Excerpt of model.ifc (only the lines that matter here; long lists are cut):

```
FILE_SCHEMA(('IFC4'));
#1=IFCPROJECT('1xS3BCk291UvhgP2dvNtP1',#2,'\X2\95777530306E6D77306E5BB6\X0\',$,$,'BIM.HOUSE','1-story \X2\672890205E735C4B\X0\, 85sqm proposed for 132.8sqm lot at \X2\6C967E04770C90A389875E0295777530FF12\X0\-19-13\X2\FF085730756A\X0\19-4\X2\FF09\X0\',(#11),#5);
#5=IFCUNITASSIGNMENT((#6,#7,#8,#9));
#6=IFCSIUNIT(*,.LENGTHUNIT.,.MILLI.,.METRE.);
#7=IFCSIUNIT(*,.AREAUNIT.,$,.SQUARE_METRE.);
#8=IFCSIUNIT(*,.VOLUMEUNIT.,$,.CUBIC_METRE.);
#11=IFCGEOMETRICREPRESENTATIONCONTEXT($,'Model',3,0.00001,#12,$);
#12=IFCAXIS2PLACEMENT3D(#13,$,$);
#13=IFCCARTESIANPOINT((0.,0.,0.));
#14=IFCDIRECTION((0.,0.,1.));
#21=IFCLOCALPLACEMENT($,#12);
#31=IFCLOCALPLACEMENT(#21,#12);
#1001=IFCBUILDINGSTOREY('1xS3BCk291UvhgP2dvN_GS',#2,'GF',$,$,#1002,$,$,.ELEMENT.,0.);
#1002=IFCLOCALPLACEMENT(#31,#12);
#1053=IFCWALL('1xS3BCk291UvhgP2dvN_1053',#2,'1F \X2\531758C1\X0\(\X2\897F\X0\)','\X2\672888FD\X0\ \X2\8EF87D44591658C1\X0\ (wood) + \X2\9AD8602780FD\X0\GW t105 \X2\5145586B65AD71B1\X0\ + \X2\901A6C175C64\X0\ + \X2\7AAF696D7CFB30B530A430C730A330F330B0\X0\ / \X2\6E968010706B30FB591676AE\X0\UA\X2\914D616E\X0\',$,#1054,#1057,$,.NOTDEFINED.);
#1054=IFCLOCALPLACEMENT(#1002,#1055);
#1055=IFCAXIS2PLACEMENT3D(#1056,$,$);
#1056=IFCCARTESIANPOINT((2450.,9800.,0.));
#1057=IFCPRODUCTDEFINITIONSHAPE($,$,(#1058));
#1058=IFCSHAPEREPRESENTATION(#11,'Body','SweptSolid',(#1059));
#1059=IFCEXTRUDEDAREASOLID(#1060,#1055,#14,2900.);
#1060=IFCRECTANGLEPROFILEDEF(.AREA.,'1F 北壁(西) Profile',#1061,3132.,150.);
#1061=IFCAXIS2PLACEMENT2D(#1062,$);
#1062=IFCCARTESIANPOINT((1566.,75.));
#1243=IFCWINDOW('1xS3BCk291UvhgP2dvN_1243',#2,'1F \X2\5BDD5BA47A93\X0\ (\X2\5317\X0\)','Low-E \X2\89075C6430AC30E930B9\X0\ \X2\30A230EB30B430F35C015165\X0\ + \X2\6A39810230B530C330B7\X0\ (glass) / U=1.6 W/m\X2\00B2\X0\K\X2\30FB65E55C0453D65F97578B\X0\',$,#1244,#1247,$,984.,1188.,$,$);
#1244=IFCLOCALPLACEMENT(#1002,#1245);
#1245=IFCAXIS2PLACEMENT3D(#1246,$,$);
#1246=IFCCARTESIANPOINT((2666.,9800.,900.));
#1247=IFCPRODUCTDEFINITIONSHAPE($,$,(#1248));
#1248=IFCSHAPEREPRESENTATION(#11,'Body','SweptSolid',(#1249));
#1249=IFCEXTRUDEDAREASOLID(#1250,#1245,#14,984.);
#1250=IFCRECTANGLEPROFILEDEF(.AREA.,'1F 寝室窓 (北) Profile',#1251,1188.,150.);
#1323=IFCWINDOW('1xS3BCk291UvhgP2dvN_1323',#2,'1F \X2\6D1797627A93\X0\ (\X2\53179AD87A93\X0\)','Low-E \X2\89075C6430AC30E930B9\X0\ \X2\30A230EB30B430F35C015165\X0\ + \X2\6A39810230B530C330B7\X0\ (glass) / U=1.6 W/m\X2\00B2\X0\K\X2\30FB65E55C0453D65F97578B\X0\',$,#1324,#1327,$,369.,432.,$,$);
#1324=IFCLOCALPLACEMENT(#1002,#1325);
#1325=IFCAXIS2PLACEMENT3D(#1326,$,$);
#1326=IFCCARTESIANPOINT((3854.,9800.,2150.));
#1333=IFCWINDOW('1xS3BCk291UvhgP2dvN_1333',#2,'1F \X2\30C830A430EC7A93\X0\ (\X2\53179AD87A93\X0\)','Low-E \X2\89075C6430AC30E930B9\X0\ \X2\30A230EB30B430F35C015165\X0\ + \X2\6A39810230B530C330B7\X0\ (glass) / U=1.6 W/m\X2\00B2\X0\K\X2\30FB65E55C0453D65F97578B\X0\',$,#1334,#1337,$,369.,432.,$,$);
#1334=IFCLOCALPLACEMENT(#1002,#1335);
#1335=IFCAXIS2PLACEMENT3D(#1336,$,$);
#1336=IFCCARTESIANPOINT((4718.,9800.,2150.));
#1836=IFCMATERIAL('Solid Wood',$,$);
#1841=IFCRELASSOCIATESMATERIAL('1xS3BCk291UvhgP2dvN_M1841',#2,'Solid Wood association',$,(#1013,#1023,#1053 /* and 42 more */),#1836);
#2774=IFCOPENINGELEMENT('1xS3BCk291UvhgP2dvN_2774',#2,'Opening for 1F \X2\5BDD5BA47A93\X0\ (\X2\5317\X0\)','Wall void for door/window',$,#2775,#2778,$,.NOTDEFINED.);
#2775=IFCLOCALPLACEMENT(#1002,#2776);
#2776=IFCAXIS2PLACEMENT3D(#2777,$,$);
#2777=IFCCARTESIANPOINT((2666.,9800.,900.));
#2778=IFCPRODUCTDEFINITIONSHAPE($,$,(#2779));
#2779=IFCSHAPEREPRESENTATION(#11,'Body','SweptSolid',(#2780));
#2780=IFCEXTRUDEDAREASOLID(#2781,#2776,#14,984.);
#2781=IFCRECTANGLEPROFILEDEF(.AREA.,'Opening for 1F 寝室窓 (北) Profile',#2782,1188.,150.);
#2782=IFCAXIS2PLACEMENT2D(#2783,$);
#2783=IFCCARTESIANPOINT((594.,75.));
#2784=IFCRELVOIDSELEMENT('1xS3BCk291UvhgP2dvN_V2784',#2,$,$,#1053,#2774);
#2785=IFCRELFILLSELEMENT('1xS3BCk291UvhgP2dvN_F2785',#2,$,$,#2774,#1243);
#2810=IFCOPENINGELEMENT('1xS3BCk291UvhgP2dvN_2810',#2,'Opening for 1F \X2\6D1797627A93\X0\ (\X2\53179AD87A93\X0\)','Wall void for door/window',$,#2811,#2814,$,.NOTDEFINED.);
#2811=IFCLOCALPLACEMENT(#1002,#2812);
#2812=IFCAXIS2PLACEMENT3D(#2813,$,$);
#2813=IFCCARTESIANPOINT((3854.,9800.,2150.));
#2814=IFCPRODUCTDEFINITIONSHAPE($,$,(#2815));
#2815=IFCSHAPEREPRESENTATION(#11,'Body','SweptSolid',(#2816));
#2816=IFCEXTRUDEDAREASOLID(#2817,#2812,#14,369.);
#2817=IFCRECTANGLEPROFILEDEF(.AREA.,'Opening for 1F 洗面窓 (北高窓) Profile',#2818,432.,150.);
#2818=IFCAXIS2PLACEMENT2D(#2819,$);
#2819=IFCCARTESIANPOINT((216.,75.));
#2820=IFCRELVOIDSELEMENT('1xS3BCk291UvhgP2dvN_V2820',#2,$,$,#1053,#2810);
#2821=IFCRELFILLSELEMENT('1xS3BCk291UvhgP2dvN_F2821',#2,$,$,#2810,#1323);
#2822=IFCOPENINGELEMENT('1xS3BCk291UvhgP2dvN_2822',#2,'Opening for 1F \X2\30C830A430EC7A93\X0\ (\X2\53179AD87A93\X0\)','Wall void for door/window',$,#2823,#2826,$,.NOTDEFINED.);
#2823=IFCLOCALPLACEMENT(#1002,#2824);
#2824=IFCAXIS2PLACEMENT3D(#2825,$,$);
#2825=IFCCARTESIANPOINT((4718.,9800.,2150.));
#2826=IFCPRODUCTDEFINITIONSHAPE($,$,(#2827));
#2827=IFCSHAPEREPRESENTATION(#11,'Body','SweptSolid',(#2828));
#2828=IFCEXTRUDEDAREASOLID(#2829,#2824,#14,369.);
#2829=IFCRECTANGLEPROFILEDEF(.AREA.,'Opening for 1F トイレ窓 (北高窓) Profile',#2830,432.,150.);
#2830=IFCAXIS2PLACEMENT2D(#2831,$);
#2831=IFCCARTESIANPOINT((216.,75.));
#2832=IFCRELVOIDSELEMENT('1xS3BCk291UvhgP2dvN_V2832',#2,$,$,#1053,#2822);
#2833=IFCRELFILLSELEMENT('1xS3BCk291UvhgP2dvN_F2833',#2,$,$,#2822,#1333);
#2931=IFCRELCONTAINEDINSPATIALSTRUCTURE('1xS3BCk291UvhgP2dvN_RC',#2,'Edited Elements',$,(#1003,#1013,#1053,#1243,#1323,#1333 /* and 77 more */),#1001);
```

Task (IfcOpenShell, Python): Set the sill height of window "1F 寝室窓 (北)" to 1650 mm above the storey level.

```python
import numpy as np
import ifcopenshell
import ifcopenshell.api.geometry
import ifcopenshell.geom
import ifcopenshell.util.element
import ifcopenshell.util.placement
import ifcopenshell.util.shape
import ifcopenshell.util.unit

model = ifcopenshell.open("model.ifc")
unit_scale = ifcopenshell.util.unit.calculate_unit_scale(model)

window = model.by_guid("1xS3BCk291UvhgP2dvN_1243")
opening = window.FillsVoids[0].RelatingOpeningElement
storey = ifcopenshell.util.element.get_container(window, ifc_class="IfcBuildingStorey")
level = ifcopenshell.util.placement.get_local_placement(storey.ObjectPlacement)[2, 3]

# The opening's origin need not be at the sill, so measure its lowest point.
shape = ifcopenshell.geom.create_shape(ifcopenshell.geom.settings(), opening)
bottom = ifcopenshell.util.shape.get_shape_bottom_elevation(shape, shape.geometry) / unit_scale
dz = level + 1.65 / unit_scale - bottom

shift = np.array([0.0, 0.0, dz])
# The window is not placed relative to its opening, so move both.
for product in (opening, window):
    matrix = ifcopenshell.util.placement.get_local_placement(product.ObjectPlacement)
    matrix[:3, 3] += shift
    ifcopenshell.api.geometry.edit_object_placement(model, product=product, matrix=matrix, is_si=False)

print(f"moved by {dz * unit_scale:+.3f} m")

model.write("model_updated.ifc")
```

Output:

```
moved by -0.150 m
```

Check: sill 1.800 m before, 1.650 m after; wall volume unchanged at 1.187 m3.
